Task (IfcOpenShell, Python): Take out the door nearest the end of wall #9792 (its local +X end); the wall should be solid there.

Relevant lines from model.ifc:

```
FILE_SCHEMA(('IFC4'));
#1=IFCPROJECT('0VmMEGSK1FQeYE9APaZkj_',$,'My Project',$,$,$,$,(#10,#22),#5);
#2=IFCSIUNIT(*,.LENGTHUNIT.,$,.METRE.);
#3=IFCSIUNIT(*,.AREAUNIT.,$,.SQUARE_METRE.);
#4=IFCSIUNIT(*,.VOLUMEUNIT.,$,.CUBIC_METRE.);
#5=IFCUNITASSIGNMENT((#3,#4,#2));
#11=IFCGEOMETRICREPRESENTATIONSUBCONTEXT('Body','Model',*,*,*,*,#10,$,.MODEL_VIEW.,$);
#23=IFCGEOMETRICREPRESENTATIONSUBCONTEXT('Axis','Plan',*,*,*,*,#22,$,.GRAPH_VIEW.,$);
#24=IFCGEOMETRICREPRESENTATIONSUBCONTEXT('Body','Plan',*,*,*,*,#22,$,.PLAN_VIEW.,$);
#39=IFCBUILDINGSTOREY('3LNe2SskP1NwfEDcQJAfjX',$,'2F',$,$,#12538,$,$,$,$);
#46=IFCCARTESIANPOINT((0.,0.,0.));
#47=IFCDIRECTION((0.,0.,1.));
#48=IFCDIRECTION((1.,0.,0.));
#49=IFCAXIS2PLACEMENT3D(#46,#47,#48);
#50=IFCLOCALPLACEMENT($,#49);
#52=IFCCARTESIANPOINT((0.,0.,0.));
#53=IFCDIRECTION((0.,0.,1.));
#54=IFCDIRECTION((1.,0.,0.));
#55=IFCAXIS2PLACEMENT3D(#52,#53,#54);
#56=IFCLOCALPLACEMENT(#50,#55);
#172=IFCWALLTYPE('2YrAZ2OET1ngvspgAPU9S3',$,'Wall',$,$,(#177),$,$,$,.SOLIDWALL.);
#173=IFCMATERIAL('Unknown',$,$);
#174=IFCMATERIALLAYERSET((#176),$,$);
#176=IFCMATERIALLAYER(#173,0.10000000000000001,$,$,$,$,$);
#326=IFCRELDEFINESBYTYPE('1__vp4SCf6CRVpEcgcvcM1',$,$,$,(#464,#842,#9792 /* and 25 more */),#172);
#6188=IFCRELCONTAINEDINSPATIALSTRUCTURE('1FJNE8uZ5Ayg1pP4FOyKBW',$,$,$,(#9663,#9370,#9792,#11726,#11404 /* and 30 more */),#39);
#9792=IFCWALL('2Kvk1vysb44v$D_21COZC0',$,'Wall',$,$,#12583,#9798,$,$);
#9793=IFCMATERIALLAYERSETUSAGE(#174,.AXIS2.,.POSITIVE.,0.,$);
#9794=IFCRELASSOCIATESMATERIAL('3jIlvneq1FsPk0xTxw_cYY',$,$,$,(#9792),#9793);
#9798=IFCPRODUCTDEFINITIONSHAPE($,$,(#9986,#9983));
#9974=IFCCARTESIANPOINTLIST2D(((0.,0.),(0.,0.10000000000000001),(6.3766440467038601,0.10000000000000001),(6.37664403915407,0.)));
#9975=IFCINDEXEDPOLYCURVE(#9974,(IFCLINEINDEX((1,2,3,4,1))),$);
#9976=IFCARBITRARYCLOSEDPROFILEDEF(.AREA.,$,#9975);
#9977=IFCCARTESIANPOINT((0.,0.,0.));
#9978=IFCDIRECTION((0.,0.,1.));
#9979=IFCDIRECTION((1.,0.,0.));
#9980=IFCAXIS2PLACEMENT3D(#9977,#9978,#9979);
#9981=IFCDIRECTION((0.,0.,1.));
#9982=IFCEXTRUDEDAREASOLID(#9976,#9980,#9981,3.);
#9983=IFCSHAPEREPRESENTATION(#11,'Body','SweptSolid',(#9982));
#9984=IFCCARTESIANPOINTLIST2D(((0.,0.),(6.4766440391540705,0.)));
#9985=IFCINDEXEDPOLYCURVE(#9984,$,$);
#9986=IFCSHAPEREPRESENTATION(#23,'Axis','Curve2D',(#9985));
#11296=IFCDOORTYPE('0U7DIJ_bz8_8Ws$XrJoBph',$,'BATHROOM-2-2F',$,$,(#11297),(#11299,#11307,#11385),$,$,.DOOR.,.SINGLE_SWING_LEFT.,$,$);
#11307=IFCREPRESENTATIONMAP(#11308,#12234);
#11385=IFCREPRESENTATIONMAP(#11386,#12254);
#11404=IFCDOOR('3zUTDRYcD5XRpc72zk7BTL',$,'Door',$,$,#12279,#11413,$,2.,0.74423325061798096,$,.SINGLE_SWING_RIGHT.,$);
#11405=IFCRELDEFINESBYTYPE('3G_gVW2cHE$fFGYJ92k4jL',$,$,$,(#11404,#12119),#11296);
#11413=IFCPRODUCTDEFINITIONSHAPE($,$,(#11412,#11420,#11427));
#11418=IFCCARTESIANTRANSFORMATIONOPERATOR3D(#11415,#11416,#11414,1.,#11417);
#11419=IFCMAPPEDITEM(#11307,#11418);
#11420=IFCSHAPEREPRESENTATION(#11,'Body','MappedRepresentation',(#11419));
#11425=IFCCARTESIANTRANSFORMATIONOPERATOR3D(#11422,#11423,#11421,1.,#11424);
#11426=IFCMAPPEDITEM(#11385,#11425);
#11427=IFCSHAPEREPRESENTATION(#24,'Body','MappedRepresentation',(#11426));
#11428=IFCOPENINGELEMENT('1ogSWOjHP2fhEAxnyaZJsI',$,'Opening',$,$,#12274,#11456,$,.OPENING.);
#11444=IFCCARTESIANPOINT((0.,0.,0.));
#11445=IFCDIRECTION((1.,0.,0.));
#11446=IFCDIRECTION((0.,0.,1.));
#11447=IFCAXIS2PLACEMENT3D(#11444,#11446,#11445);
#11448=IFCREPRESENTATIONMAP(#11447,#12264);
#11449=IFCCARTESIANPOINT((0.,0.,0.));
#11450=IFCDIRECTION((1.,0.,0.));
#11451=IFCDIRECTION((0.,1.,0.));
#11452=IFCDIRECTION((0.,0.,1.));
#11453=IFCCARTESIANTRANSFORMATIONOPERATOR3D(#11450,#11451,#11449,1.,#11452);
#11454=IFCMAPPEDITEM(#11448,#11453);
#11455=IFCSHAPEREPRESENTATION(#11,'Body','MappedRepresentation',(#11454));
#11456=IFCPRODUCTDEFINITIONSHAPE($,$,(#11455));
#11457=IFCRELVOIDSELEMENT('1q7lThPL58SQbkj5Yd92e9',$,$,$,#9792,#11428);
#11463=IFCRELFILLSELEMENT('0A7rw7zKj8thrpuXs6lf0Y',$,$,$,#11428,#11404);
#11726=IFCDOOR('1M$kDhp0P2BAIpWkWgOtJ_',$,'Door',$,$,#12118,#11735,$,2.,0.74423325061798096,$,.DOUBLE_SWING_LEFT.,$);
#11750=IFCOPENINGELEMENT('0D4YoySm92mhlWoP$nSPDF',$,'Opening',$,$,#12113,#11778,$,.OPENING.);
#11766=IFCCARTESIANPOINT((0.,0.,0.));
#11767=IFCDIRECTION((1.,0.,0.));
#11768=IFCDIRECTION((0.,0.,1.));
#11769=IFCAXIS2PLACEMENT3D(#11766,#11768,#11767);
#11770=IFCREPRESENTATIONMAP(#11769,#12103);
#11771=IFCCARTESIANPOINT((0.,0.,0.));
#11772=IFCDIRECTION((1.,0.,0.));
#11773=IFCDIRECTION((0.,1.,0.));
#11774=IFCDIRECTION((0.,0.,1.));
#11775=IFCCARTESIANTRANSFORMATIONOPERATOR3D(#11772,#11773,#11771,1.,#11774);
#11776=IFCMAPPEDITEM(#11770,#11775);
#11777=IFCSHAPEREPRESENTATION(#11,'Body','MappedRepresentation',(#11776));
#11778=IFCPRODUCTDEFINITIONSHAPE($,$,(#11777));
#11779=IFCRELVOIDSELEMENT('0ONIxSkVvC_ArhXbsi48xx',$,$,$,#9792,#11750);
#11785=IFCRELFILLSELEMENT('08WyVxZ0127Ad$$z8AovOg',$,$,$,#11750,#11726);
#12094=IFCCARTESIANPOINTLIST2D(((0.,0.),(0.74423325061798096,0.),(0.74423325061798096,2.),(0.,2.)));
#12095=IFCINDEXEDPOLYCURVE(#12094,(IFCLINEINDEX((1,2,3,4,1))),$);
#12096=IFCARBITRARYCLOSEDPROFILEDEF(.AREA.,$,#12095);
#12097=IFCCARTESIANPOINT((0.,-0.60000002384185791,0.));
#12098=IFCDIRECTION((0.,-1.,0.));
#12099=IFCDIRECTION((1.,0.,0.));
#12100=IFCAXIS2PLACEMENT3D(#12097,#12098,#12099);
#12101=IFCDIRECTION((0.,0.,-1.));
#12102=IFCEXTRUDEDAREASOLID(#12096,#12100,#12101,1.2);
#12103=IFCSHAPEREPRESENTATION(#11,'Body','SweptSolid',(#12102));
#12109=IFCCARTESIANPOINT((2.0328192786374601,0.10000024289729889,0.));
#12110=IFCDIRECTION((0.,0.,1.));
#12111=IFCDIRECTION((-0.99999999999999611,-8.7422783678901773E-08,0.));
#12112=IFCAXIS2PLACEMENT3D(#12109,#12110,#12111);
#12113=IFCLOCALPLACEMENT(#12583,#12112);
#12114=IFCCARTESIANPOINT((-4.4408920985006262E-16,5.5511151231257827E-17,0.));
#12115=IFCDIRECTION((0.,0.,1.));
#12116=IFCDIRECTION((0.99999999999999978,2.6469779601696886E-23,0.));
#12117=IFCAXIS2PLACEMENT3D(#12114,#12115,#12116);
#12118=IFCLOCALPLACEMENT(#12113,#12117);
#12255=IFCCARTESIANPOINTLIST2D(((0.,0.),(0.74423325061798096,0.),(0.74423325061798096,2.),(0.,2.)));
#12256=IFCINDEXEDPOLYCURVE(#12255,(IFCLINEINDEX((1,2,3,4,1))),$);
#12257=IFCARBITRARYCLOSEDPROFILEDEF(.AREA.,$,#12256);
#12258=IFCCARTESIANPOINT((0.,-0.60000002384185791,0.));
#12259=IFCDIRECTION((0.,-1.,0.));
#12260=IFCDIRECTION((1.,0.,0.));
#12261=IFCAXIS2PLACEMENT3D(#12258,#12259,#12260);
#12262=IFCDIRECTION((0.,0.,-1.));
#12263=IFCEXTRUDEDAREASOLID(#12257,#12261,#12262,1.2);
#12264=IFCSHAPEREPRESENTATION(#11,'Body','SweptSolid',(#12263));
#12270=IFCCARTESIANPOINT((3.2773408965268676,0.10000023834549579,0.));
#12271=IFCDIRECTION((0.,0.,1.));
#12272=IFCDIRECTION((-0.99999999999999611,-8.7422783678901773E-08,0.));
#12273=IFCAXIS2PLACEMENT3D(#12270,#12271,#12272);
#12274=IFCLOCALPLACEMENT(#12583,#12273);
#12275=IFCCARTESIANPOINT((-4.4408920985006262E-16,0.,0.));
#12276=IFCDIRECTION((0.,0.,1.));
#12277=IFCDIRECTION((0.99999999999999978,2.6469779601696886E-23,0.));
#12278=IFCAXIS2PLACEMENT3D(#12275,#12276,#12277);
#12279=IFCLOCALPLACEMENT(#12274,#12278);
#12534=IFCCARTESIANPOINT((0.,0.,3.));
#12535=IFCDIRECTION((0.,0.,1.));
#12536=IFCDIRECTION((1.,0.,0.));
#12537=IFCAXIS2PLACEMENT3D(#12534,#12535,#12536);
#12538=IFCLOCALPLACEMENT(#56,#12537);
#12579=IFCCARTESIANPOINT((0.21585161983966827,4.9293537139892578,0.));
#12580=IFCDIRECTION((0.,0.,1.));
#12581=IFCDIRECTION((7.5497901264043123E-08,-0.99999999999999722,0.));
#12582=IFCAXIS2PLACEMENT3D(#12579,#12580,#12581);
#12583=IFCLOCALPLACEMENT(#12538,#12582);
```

```python
import ifcopenshell
import ifcopenshell.api.feature
import ifcopenshell.api.root
import ifcopenshell.geom
import ifcopenshell.util.shape

model = ifcopenshell.open("model.ifc")
settings = ifcopenshell.geom.settings()


def volume(element):
    """Net volume in cubic metres, openings subtracted."""
    shape = ifcopenshell.geom.create_shape(settings, element)
    return ifcopenshell.util.shape.get_volume(shape.geometry)


door = model.by_guid("3zUTDRYcD5XRpc72zk7BTL")
opening = door.FillsVoids[0].RelatingOpeningElement
wall = opening.VoidsElements[0].RelatingBuildingElement
before = volume(wall)

ifcopenshell.api.root.remove_product(model, product=door)
ifcopenshell.api.feature.remove_feature(model, feature=opening)

after = volume(wall)

print(f"wall volume {before:.3f} -> {after:.3f} m3")

model.write("model_edited.ifc")
```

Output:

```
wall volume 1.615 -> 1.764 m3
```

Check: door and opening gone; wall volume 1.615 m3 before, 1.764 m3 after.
